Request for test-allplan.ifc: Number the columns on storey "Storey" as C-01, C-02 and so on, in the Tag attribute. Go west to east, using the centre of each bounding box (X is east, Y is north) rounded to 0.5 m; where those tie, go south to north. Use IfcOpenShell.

First a look at what the model holds.

```python
import ifcopenshell
import ifcopenshell.util.element
import ifcopenshell.util.placement

model = ifcopenshell.open("test-allplan.ifc")
print(model.schema)
storey = next(s for s in model.by_type("IfcBuildingStorey") if s.Name == "Storey")
columns = [e for e in ifcopenshell.util.element.get_decomposition(storey) if e.is_a("IfcColumn")]
for e in sorted(columns, key=lambda e: e.id()):
    origin = ifcopenshell.util.placement.get_local_placement(e.ObjectPlacement)[:3, 3]
    print(e.id(), e.Tag, e.Name, origin.round(2) + 0.0, sep=" | ")
```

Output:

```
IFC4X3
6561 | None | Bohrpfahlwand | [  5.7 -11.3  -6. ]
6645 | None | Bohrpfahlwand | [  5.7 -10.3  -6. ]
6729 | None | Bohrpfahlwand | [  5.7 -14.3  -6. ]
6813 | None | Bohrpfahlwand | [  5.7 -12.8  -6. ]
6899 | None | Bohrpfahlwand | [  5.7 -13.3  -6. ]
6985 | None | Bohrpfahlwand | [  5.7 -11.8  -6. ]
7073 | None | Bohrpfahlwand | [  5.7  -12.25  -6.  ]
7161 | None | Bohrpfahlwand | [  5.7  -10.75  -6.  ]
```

```python
import ifcopenshell
import ifcopenshell.geom
import ifcopenshell.util.element
import ifcopenshell.util.shape

model = ifcopenshell.open("test-allplan.ifc")
settings = ifcopenshell.geom.settings()
settings.set("use-world-coords", True)


def centre(element):
    shape = ifcopenshell.geom.create_shape(settings, element)
    return ifcopenshell.util.shape.get_bbox_centroid(shape.geometry)


storey = next(s for s in model.by_type("IfcBuildingStorey") if s.Name == "Storey")
columns = [e for e in ifcopenshell.util.element.get_decomposition(storey) if e.is_a("IfcColumn")]

# Insertion points can sit at a corner or the storey origin, so sort by the geometry (in metres).
centres = {e: centre(e) for e in columns}
columns.sort(key=lambda e: (round(centres[e][0] / 0.5), centres[e][1]))

for i, e in enumerate(columns, start=1):
    number = f"C-{i:02d}"
    e.Tag = number
    print(e.id(), number)

model.write("test-allplan_updated.ifc")
```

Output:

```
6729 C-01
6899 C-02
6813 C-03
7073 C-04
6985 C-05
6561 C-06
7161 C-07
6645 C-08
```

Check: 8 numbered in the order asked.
